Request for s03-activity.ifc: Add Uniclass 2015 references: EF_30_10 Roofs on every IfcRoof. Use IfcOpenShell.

First a look at what the model holds.

```python
import ifcopenshell

model = ifcopenshell.open("s03-activity.ifc")
print(model.schema)
print("classifications:", [c.Name for c in model.by_type("IfcClassification")])
for ifc_class in ("IfcDoor", "IfcRoof", "IfcStair", "IfcWall", "IfcWindow"):
    print(ifc_class, len(model.by_type(ifc_class)))
```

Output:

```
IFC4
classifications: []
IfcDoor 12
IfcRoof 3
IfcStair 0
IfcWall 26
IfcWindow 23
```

```python
import ifcopenshell
import ifcopenshell.api.classification

model = ifcopenshell.open("s03-activity.ifc")

system = ifcopenshell.api.classification.add_classification(model, classification="Uniclass 2015")

codes = {
    "IfcRoof": ("EF_30_10", "Roofs"),
}
for ifc_class, (code, name) in codes.items():
    products = model.by_type(ifc_class)
    ifcopenshell.api.classification.add_reference(
        model, products=products, classification=system, identification=code, name=name
    )
    print(code, len(products))

model.write("s03-activity_edited.ifc")
```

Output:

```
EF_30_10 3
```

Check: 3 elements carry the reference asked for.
